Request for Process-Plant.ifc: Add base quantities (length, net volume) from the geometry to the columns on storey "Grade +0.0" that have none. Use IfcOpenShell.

First a look at what the model holds.

```python
import ifcopenshell
import ifcopenshell.util.element
import ifcopenshell.util.unit

model = ifcopenshell.open("Process-Plant.ifc")
print(model.schema)
for unit_type in ("LENGTHUNIT", "AREAUNIT", "VOLUMEUNIT"):
    print(unit_type, ifcopenshell.util.unit.calculate_unit_scale(model, unit_type))
storey = next(s for s in model.by_type("IfcBuildingStorey") if s.Name == "Grade +0.0")
columns = [e for e in ifcopenshell.util.element.get_decomposition(storey) if e.is_a("IfcColumn")]
for e in sorted(columns, key=lambda e: e.id()):
    print(e.id(), e.is_a(), e.Name, list(ifcopenshell.util.element.get_psets(e, qtos_only=True)), sep=" | ")
```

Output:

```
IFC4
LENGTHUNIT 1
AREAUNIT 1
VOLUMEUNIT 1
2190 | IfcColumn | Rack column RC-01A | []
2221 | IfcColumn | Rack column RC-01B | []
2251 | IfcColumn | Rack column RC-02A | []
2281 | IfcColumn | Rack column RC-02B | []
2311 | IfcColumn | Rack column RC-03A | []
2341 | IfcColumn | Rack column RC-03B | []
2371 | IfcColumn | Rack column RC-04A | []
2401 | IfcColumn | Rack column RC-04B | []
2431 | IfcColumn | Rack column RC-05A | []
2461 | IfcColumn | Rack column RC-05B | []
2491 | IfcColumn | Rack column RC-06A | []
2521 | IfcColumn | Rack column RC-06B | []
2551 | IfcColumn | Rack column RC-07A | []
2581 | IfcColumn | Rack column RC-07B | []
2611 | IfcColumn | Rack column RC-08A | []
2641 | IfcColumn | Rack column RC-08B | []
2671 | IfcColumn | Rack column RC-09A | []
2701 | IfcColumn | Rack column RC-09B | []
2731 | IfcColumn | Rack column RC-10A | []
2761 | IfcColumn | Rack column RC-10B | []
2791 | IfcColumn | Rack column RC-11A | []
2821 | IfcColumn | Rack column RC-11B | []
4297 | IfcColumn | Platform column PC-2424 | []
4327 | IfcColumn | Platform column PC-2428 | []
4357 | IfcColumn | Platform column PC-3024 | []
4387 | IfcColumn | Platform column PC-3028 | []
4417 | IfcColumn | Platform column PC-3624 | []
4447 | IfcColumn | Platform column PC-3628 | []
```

```python
import ifcopenshell
import ifcopenshell.api.pset
import ifcopenshell.geom
import ifcopenshell.util.element
import ifcopenshell.util.shape
import ifcopenshell.util.unit

model = ifcopenshell.open("Process-Plant.ifc")
unit_scale = ifcopenshell.util.unit.calculate_unit_scale(model)
volume_scale = ifcopenshell.util.unit.calculate_unit_scale(model, "VOLUMEUNIT")
settings = ifcopenshell.geom.settings()

storey = next(s for s in model.by_type("IfcBuildingStorey") if s.Name == "Grade +0.0")
columns = [e for e in ifcopenshell.util.element.get_decomposition(storey) if e.is_a("IfcColumn")]

for e in sorted(columns, key=lambda e: e.id()):
    if ifcopenshell.util.element.get_psets(e, qtos_only=True, should_inherit=False):
        continue
    # Geometry comes back in metres, in the element's own axes.
    shape = ifcopenshell.geom.create_shape(settings, e)
    values = {
        "Length": ifcopenshell.util.shape.get_z(shape.geometry) / unit_scale,
        "NetVolume": ifcopenshell.util.shape.get_volume(shape.geometry) / volume_scale,
    }
    qto = ifcopenshell.api.pset.add_qto(model, product=e, name="Qto_ColumnBaseQuantities")
    ifcopenshell.api.pset.edit_qto(model, qto=qto, properties=values)
    print(e.id(), {k: round(v, 3) for k, v in values.items()})

model.write("Process-Plant_edited.ifc")
```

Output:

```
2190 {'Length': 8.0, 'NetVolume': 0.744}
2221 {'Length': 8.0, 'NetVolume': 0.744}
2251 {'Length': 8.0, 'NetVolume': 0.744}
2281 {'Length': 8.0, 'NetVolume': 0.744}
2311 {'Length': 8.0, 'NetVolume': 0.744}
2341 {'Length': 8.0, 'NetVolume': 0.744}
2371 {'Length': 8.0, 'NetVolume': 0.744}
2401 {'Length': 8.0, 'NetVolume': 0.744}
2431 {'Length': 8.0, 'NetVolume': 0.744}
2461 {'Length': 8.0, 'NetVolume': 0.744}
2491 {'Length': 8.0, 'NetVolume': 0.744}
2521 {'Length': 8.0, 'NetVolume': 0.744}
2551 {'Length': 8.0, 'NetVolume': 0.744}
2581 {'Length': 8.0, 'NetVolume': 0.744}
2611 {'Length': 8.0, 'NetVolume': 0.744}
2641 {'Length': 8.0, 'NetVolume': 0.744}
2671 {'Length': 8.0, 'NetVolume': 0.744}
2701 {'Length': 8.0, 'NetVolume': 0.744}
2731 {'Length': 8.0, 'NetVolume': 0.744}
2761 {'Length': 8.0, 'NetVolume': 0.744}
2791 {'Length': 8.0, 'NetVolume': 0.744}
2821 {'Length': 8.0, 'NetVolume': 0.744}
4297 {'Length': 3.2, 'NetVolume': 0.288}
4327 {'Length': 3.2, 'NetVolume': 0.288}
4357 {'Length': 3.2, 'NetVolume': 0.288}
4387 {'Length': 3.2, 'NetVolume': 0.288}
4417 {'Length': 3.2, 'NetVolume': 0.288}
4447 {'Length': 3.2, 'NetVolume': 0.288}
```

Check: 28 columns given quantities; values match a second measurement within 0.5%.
